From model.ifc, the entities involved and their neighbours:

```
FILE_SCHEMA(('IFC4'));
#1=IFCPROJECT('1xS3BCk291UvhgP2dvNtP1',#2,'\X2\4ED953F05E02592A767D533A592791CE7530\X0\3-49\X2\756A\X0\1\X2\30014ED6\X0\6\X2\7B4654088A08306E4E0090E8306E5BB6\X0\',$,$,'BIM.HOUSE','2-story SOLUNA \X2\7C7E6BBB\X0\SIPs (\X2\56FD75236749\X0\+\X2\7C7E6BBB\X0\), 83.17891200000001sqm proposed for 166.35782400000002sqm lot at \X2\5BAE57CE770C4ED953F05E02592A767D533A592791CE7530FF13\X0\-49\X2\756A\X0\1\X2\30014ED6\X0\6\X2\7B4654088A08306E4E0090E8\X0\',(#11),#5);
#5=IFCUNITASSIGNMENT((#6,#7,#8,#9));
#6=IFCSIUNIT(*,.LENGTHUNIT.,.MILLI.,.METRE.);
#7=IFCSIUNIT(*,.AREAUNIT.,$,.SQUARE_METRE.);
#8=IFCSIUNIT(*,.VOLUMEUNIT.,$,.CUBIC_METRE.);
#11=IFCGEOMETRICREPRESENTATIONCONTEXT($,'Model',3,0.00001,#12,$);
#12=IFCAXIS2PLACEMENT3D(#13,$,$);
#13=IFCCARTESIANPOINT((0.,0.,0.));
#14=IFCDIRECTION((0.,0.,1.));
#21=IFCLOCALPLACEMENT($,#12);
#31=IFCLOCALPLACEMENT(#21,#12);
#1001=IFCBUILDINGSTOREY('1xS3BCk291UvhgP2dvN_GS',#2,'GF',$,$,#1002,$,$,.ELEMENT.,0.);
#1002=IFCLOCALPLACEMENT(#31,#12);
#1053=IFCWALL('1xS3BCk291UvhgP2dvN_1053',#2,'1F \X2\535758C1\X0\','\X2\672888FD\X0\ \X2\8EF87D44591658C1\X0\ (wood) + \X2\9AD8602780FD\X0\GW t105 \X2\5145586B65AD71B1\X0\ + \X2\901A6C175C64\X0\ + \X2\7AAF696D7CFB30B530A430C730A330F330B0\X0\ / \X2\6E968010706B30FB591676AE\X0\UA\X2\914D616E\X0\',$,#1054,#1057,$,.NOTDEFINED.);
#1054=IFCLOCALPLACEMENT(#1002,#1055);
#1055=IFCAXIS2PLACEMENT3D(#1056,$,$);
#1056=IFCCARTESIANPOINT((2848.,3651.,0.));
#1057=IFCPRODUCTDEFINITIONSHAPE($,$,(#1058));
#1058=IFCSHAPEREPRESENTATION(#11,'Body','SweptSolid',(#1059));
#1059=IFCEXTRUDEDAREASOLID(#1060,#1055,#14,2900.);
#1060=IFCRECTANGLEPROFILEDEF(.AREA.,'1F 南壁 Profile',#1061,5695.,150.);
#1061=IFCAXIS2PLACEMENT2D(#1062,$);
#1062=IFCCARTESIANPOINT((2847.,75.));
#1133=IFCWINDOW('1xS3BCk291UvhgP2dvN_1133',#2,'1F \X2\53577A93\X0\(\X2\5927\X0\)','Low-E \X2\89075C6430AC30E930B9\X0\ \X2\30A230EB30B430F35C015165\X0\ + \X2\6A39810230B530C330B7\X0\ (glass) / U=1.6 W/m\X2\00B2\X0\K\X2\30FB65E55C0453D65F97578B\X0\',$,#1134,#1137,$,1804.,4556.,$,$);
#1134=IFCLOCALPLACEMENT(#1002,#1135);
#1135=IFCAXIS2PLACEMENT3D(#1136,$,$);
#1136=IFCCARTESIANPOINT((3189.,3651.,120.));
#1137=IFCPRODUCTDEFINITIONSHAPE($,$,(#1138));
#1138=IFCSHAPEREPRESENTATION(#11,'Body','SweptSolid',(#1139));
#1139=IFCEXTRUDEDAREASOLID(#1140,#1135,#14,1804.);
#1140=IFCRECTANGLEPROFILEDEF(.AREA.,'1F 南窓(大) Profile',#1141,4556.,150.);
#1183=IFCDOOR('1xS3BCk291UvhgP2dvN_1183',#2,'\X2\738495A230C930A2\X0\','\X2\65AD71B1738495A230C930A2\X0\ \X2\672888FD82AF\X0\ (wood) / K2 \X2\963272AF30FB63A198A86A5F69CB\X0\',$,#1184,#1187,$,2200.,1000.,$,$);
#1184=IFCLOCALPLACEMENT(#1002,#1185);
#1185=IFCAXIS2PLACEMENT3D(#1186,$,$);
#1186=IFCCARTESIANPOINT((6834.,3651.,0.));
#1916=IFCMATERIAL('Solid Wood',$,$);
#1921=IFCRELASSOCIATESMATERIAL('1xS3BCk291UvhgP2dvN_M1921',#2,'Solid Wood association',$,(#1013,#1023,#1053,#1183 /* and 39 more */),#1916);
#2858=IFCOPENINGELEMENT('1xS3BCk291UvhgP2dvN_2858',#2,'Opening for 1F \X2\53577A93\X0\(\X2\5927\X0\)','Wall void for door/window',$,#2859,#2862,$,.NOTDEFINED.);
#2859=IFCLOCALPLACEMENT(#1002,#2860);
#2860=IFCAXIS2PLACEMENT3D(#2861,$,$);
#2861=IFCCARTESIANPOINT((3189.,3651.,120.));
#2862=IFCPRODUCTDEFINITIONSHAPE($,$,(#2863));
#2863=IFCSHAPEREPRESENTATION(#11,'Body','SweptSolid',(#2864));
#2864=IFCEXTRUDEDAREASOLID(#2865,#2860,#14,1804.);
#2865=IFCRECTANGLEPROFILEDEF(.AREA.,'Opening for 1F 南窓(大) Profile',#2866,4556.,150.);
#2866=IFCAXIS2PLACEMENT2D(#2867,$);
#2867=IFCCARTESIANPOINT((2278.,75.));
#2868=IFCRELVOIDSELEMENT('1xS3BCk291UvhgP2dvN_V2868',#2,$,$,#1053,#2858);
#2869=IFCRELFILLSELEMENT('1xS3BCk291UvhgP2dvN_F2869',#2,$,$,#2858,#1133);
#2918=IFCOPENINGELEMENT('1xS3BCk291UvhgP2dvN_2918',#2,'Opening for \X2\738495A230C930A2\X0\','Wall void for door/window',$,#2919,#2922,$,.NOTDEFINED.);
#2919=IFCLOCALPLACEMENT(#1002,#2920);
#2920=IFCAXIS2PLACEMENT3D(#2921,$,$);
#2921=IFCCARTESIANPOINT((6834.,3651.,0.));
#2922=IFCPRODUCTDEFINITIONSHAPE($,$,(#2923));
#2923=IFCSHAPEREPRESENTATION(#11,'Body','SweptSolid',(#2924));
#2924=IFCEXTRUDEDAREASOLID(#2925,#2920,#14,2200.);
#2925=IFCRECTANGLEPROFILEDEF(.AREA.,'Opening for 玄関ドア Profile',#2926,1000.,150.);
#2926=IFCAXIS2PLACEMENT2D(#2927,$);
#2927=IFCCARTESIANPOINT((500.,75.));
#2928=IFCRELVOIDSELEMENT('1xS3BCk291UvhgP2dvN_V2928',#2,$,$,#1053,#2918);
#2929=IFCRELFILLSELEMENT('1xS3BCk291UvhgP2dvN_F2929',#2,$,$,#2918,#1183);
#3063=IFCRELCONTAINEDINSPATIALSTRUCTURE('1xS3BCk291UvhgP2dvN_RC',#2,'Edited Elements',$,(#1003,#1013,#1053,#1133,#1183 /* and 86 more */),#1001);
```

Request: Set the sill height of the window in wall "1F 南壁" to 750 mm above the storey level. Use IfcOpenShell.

```python
import numpy as np
import ifcopenshell
import ifcopenshell.api.geometry
import ifcopenshell.geom
import ifcopenshell.util.element
import ifcopenshell.util.placement
import ifcopenshell.util.shape
import ifcopenshell.util.unit

model = ifcopenshell.open("model.ifc")
unit_scale = ifcopenshell.util.unit.calculate_unit_scale(model)

window = model.by_id(1133)
opening = window.FillsVoids[0].RelatingOpeningElement
storey = ifcopenshell.util.element.get_container(window, ifc_class="IfcBuildingStorey")
level = ifcopenshell.util.placement.get_local_placement(storey.ObjectPlacement)[2, 3]

# The opening's origin need not be at the sill, so measure its lowest point.
shape = ifcopenshell.geom.create_shape(ifcopenshell.geom.settings(), opening)
bottom = ifcopenshell.util.shape.get_shape_bottom_elevation(shape, shape.geometry) / unit_scale
dz = level + 0.75 / unit_scale - bottom

shift = np.array([0.0, 0.0, dz])
# The window is not placed relative to its opening, so move both.
for product in (opening, window):
    matrix = ifcopenshell.util.placement.get_local_placement(product.ObjectPlacement)
    matrix[:3, 3] += shift
    ifcopenshell.api.geometry.edit_object_placement(model, product=product, matrix=matrix, is_si=False)

print(f"moved by {dz * unit_scale:+.3f} m")

model.write("model_updated.ifc")
```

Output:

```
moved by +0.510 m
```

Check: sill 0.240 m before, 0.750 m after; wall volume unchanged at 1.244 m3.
